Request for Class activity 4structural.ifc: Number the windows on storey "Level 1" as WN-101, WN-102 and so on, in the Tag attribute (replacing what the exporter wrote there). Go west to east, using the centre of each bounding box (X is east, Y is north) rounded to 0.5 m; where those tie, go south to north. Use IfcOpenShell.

First a look at what the model holds.

```python
import ifcopenshell
import ifcopenshell.util.element
import ifcopenshell.util.placement

model = ifcopenshell.open("Class activity 4structural.ifc")
print(model.schema)
storey = next(s for s in model.by_type("IfcBuildingStorey") if s.Name == "Level 1")
windows = [e for e in ifcopenshell.util.element.get_decomposition(storey) if e.is_a("IfcWindow")]
for e in sorted(windows, key=lambda e: e.id()):
    origin = ifcopenshell.util.placement.get_local_placement(e.ObjectPlacement)[:3, 3]
    print(e.id(), e.Tag, e.Name, origin.round(2) + 0.0, sep=" | ")
```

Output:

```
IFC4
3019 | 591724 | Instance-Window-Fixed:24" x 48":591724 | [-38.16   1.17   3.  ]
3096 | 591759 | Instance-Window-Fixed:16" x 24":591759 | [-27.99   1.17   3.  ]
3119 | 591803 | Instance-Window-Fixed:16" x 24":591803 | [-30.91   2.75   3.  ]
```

```python
import ifcopenshell
import ifcopenshell.geom
import ifcopenshell.util.element
import ifcopenshell.util.shape

model = ifcopenshell.open("Class activity 4structural.ifc")
settings = ifcopenshell.geom.settings()
settings.set("use-world-coords", True)


def centre(element):
    shape = ifcopenshell.geom.create_shape(settings, element)
    return ifcopenshell.util.shape.get_bbox_centroid(shape.geometry)


storey = next(s for s in model.by_type("IfcBuildingStorey") if s.Name == "Level 1")
windows = [e for e in ifcopenshell.util.element.get_decomposition(storey) if e.is_a("IfcWindow")]

# Insertion points can sit at a corner or the storey origin, so sort by the geometry (in metres).
centres = {e: centre(e) for e in windows}
windows.sort(key=lambda e: (round(centres[e][0] / 0.5), centres[e][1]))

for i, e in enumerate(windows, start=1):
    number = f"WN-1{i:02d}"
    e.Tag = number
    print(e.id(), number)

model.write("Class activity 4structural_rev.ifc")
```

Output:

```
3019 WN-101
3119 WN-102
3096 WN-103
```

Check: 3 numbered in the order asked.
